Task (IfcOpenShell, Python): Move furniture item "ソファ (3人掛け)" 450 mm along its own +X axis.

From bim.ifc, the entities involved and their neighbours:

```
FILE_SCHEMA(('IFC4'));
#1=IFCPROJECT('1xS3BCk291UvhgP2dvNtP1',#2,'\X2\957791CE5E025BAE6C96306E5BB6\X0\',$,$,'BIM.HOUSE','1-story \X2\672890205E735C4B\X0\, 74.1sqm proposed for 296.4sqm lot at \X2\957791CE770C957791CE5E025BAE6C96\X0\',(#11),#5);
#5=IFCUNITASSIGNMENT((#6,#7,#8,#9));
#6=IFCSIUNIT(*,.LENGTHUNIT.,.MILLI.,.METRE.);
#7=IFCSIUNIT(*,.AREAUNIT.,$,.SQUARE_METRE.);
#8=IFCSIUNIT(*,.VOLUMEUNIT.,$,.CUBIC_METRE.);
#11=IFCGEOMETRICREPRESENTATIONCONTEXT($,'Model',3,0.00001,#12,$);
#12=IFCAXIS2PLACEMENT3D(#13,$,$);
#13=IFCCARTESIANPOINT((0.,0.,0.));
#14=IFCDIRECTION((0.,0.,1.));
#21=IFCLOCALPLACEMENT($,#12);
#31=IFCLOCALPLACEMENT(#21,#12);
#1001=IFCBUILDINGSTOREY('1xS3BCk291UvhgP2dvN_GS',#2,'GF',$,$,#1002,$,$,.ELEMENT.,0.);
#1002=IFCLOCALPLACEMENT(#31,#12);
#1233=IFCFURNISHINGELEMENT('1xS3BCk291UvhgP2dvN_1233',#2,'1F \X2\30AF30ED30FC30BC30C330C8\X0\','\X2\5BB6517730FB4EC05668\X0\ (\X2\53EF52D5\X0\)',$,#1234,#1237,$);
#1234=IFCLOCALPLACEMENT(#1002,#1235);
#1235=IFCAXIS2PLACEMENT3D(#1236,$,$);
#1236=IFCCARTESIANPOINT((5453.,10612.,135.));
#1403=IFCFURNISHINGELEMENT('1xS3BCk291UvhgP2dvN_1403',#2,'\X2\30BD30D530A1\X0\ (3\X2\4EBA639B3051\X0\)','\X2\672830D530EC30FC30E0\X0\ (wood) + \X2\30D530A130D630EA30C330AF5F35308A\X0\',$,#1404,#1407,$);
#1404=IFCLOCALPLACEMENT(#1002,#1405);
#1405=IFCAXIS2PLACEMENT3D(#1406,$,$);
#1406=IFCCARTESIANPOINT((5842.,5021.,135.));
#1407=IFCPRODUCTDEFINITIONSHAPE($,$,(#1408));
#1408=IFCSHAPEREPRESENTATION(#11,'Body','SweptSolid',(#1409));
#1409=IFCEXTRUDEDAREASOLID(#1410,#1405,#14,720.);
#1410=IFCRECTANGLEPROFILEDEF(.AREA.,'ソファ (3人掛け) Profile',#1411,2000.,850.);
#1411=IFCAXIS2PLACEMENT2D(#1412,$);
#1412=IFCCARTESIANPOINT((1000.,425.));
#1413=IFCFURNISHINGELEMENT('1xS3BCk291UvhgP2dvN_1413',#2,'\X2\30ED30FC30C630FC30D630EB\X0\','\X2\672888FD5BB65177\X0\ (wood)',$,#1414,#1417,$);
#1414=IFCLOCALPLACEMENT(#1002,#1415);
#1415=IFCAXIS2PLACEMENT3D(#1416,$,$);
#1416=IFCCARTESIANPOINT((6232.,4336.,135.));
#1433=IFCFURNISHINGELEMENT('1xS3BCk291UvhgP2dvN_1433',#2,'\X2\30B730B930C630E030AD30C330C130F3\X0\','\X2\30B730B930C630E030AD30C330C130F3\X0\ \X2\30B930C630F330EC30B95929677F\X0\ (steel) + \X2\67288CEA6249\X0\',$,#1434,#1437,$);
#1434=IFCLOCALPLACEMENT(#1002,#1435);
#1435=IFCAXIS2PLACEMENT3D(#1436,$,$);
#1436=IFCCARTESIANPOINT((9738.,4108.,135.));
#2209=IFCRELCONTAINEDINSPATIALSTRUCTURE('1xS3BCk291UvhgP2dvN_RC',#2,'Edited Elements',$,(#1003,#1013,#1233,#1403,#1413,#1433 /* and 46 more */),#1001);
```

```python
import ifcopenshell
import ifcopenshell.api.geometry
import ifcopenshell.util.placement

model = ifcopenshell.open("bim.ifc")

item = model.by_guid("1xS3BCk291UvhgP2dvN_1403")
matrix = ifcopenshell.util.placement.get_local_placement(item.ObjectPlacement)
matrix[:3, 3] += matrix[:3, 0] * 450.0
ifcopenshell.api.geometry.edit_object_placement(model, product=item, matrix=matrix, is_si=False)

print(ifcopenshell.util.placement.get_local_placement(item.ObjectPlacement).round(3) + 0.0)

model.write("bim_edited.ifc")
```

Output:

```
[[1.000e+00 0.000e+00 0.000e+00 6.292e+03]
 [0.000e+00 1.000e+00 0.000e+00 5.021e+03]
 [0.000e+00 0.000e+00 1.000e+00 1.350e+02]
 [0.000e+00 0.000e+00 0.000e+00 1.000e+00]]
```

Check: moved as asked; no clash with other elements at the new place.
